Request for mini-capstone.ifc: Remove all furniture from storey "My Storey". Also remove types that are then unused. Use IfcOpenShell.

First a look at what the model holds.

```python
import ifcopenshell
import ifcopenshell.util.element

model = ifcopenshell.open("mini-capstone.ifc")
print(model.schema)
storey = next(s for s in model.by_type("IfcBuildingStorey") if s.Name == "My Storey")
furniture = [e for e in ifcopenshell.util.element.get_decomposition(storey) if e.is_a("IfcFurnishingElement")]
seen = {}
for e in furniture:
    element_type = ifcopenshell.util.element.get_type(e)
    name = element_type.Name if element_type not in (None, e) else None
    seen[name] = seen.get(name, 0) + 1
for name, count in sorted(seen.items(), key=str):
    print(count, "x", name)
```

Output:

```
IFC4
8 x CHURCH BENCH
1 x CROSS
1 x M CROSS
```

```python
import ifcopenshell
import ifcopenshell.api.root
import ifcopenshell.util.element

model = ifcopenshell.open("mini-capstone.ifc")

storey = next(s for s in model.by_type("IfcBuildingStorey") if s.Name == "My Storey")
furniture = [e for e in ifcopenshell.util.element.get_decomposition(storey) if e.is_a("IfcFurnishingElement")]
types = {ifcopenshell.util.element.get_type(e) for e in furniture} - {None, *furniture}

for e in furniture:
    ifcopenshell.api.root.remove_product(model, product=e)
print(len(furniture), "removed")

unused = [t for t in types if not ifcopenshell.util.element.get_types(t)]
for t in unused:
    ifcopenshell.api.root.remove_product(model, product=t)
print(len(unused), "unused types removed")

model.write("mini-capstone_edited.ifc")
```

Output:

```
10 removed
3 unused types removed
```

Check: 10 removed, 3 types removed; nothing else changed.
